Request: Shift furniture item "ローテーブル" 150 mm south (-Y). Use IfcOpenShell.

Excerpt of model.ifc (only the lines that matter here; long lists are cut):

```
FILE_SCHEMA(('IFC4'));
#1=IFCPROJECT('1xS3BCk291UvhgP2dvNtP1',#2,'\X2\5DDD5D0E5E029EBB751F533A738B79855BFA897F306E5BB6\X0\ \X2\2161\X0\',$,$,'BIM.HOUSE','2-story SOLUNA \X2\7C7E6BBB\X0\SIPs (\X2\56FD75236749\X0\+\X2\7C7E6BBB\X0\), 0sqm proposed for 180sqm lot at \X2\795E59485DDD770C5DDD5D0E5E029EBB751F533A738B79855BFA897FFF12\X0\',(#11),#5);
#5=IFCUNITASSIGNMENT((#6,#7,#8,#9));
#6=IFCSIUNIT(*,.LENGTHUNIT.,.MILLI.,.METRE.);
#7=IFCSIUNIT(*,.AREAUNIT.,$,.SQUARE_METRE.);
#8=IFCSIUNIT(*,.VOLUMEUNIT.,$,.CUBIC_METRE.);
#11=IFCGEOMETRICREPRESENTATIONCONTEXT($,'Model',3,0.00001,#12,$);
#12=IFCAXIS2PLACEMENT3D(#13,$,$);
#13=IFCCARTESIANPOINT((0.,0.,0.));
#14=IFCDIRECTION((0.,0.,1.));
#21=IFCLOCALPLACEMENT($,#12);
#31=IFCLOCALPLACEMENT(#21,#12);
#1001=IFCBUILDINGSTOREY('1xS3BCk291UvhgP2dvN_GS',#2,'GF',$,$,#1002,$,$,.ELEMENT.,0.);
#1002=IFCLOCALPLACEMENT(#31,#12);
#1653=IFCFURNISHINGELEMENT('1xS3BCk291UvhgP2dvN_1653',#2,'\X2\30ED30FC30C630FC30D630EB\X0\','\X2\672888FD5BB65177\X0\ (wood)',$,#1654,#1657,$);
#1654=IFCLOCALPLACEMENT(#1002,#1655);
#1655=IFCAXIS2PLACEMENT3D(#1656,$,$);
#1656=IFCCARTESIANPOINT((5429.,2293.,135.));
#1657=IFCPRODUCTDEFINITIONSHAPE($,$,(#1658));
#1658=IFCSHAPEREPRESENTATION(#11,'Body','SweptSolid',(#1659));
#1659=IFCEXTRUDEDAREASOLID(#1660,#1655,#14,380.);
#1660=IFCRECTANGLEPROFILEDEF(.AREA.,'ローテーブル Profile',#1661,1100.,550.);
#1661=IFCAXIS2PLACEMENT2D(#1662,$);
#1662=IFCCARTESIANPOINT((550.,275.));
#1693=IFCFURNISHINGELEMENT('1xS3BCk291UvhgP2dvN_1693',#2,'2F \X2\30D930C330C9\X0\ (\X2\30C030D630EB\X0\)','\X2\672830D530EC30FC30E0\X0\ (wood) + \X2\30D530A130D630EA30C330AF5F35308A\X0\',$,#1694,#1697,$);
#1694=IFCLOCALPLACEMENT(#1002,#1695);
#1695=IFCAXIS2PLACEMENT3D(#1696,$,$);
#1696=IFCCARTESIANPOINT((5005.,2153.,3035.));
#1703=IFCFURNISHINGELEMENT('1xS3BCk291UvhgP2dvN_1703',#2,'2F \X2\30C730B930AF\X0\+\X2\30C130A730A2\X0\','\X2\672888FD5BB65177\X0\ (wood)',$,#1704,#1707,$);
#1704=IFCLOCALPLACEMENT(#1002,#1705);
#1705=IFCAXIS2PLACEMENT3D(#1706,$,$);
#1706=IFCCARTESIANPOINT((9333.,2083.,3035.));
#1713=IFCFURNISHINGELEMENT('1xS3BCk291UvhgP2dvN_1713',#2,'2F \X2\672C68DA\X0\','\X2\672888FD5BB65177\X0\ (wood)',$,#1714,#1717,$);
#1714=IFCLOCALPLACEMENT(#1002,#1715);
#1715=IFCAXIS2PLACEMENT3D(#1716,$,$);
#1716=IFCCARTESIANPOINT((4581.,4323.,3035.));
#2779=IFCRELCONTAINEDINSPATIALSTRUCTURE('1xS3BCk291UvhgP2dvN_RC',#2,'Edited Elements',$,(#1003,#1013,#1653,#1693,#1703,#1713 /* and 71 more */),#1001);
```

```python
import ifcopenshell
import ifcopenshell.api.geometry
import ifcopenshell.util.placement
import ifcopenshell.util.unit

model = ifcopenshell.open("model.ifc")
unit_scale = ifcopenshell.util.unit.calculate_unit_scale(model)

item = model.by_guid("1xS3BCk291UvhgP2dvN_1653")
matrix = ifcopenshell.util.placement.get_local_placement(item.ObjectPlacement)
matrix[1, 3] -= 0.15 / unit_scale
ifcopenshell.api.geometry.edit_object_placement(model, product=item, matrix=matrix, is_si=False)

print(ifcopenshell.util.placement.get_local_placement(item.ObjectPlacement).round(3) + 0.0)

model.write("model_edited.ifc")
```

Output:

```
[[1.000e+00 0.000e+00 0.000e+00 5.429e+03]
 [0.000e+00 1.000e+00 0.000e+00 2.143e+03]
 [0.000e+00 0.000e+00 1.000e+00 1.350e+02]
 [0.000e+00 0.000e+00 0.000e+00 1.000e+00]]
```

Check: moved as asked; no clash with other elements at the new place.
